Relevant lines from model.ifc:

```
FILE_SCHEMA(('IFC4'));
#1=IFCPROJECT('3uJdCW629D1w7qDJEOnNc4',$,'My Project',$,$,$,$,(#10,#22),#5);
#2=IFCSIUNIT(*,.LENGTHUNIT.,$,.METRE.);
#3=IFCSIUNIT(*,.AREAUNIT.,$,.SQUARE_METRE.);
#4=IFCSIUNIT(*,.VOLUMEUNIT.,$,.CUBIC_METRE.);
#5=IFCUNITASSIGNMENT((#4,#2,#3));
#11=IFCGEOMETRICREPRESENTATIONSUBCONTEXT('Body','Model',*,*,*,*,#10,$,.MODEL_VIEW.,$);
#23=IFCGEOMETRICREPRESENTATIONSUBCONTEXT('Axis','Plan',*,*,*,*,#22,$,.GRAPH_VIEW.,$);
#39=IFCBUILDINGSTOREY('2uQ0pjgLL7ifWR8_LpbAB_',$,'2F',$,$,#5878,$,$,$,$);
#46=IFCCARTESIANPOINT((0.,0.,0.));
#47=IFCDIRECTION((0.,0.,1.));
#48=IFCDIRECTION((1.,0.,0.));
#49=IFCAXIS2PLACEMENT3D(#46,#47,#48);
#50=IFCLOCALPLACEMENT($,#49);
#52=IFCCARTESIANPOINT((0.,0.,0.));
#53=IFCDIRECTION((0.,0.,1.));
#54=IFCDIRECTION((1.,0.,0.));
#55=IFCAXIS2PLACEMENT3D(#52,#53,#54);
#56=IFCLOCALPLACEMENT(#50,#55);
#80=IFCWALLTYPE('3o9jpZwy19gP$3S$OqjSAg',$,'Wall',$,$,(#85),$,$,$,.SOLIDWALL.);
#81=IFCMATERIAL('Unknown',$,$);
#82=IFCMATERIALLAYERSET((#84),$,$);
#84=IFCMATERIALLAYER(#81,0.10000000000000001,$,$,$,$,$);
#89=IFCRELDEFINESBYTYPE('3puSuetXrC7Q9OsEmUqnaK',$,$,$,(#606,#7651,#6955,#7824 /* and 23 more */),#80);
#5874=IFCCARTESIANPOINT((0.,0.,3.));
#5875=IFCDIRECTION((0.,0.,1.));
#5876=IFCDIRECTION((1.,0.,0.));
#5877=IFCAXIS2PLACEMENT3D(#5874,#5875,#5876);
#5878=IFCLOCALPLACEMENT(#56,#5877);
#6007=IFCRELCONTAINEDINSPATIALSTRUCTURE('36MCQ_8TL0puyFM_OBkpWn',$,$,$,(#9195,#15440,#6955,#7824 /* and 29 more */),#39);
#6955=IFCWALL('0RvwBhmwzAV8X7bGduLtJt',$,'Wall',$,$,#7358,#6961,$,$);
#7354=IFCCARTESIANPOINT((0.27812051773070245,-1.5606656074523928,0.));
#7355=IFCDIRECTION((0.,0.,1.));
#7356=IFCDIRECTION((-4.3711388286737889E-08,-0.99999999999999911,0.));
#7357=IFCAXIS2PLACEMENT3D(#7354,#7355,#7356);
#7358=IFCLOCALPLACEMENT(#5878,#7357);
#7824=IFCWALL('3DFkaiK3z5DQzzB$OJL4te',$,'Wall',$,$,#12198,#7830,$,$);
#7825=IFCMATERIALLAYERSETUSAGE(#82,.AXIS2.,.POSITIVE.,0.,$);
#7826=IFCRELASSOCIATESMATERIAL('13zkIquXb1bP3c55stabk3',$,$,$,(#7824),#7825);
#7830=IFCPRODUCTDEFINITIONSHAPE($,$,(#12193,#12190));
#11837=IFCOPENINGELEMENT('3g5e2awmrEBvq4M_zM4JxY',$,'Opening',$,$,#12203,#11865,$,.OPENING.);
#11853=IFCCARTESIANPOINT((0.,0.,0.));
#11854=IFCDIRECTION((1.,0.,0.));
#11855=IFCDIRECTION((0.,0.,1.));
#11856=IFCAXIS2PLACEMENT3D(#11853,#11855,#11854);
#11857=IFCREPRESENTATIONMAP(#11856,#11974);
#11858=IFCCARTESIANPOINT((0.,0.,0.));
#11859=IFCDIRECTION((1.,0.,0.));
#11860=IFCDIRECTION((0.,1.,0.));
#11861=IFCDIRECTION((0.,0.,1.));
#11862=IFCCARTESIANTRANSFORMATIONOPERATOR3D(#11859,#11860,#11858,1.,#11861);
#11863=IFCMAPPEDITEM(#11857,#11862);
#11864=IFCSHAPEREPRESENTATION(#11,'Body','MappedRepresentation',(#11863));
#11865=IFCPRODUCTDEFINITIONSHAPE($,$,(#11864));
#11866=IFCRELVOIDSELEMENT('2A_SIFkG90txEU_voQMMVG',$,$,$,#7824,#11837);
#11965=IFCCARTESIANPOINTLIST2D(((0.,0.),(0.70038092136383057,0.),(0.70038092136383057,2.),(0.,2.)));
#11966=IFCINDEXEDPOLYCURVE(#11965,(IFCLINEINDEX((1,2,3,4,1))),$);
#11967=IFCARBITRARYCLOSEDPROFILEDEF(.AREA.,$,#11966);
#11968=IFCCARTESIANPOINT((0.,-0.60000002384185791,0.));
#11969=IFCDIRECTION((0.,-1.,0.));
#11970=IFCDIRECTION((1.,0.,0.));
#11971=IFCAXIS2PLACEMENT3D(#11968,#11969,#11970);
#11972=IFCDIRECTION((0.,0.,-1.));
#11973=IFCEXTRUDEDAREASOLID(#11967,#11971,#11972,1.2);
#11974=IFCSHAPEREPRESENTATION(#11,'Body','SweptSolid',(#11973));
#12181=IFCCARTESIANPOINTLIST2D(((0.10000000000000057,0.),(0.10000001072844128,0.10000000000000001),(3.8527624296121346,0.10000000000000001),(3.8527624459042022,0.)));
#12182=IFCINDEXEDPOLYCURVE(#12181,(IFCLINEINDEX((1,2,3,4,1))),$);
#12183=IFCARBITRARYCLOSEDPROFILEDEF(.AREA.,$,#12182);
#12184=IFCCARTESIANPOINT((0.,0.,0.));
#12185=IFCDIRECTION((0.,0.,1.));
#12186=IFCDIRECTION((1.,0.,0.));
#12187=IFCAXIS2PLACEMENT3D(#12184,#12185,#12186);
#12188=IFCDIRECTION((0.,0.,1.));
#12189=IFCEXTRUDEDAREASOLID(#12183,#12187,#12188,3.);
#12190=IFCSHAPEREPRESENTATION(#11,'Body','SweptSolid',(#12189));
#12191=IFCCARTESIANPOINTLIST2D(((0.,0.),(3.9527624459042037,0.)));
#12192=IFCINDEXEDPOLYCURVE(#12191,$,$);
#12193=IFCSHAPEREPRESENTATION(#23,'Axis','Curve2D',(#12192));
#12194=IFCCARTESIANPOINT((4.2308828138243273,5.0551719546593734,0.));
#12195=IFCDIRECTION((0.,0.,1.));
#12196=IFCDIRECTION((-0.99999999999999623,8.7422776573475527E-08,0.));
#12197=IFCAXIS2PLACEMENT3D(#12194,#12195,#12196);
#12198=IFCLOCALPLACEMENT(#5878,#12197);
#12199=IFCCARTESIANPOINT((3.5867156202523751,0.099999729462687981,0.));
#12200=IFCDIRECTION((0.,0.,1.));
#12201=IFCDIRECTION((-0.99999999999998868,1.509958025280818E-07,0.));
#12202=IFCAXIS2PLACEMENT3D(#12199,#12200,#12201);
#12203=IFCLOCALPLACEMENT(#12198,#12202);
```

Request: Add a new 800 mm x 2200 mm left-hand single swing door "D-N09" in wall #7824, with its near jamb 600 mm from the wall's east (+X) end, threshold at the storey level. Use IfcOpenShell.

```python
import numpy as np
import ifcopenshell
import ifcopenshell.api.feature
import ifcopenshell.api.geometry
import ifcopenshell.api.root
import ifcopenshell.api.spatial
import ifcopenshell.geom
import ifcopenshell.util.element
import ifcopenshell.util.placement
import ifcopenshell.util.representation
import ifcopenshell.util.shape
import ifcopenshell.util.unit

model = ifcopenshell.open("model.ifc")
unit_scale = ifcopenshell.util.unit.calculate_unit_scale(model)
settings = ifcopenshell.geom.settings()


def volume(element):
    """Net volume in cubic metres, openings subtracted."""
    shape = ifcopenshell.geom.create_shape(settings, element)
    return ifcopenshell.util.shape.get_volume(shape.geometry)


wall = model.by_id(7824)
storey = ifcopenshell.util.element.get_container(wall, ifc_class="IfcBuildingStorey")
context = ifcopenshell.util.representation.get_context(model, "Model", "Body", "MODEL_VIEW")
before = volume(wall)

width, height, from_end, sill = 0.8, 2.2, 0.6, 0.0  # metres

# The wall runs along its own X axis, and the end named is its -X end.
wall_shape = ifcopenshell.geom.create_shape(settings, wall)
x, y, z = ifcopenshell.util.shape.get_vertices(wall_shape.geometry).T
start = x.min() + from_end
face, thickness = float(y.min()), float(y.max() - y.min())
wall_matrix = ifcopenshell.util.placement.get_local_placement(wall.ObjectPlacement)
level = ifcopenshell.util.placement.get_local_placement(storey.ObjectPlacement)[2, 3]


def in_wall(x, y):
    """Placement at x, y metres in the wall's axes, at sill height."""
    matrix = wall_matrix.copy()
    matrix[:, 3] = wall_matrix @ np.array([x / unit_scale, y / unit_scale, 0.0, 1.0])
    matrix[2, 3] = level + sill / unit_scale
    return matrix


# Opening: a box that overshoots both wall faces by 50 mm.
opening = ifcopenshell.api.root.create_entity(model, ifc_class="IfcOpeningElement", predefined_type="OPENING")
box = ifcopenshell.api.geometry.add_wall_representation(
    model, context=context, length=width, height=height, thickness=thickness + 0.1
)
ifcopenshell.api.geometry.assign_representation(model, product=opening, representation=box)
ifcopenshell.api.geometry.edit_object_placement(model, product=opening, matrix=in_wall(start, face - 0.05), is_si=False)
ifcopenshell.api.feature.add_feature(model, feature=opening, element=wall)

door = ifcopenshell.api.root.create_entity(model, ifc_class="IfcDoor", name="D-N09", predefined_type="DOOR")
door.OverallWidth, door.OverallHeight = width / unit_scale, height / unit_scale
door.OperationType = "SINGLE_SWING_LEFT"
body = ifcopenshell.api.geometry.add_door_representation(
    model,
    context=context,
    overall_width=door.OverallWidth,
    overall_height=door.OverallHeight,
    operation_type="SINGLE_SWING_LEFT",
    lining_properties={"LiningDepth": thickness / unit_scale, "ThresholdDepth": thickness / unit_scale},
)
ifcopenshell.api.geometry.assign_representation(model, product=door, representation=body)
ifcopenshell.api.spatial.assign_container(model, products=[door], relating_structure=storey)
ifcopenshell.api.feature.add_filling(model, opening=opening, element=door)

# The lining spans the wall, so the door starts at the wall face.
ifcopenshell.api.geometry.edit_object_placement(model, product=door, matrix=in_wall(start, face), is_si=False)

after = volume(wall)

print(f"wall volume {before:.3f} -> {after:.3f} m3")

model.write("model_v2.ifc")
```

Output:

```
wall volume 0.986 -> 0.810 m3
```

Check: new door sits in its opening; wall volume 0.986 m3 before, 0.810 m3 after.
